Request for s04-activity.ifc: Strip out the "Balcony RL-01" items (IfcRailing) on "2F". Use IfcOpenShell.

First a look at what the model holds.

```python
import ifcopenshell
import ifcopenshell.util.element

model = ifcopenshell.open("s04-activity.ifc")
print(model.schema)
storey = next(s for s in model.by_type("IfcBuildingStorey") if s.Name == "2F")
railings = [e for e in ifcopenshell.util.element.get_decomposition(storey) if e.is_a("IfcRailing")]
seen = {}
for e in railings:
    element_type = ifcopenshell.util.element.get_type(e)
    name = element_type.Name if element_type not in (None, e) else None
    seen[name] = seen.get(name, 0) + 1
for name, count in sorted(seen.items(), key=str):
    print(count, "x", name)
```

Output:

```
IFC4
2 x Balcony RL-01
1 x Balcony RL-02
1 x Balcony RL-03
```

```python
import ifcopenshell
import ifcopenshell.api.root
import ifcopenshell.util.element

model = ifcopenshell.open("s04-activity.ifc")

storey = next(s for s in model.by_type("IfcBuildingStorey") if s.Name == "2F")
railings = [e for e in ifcopenshell.util.element.get_decomposition(storey) if e.is_a("IfcRailing")]
targets = [e for e in railings if (t := ifcopenshell.util.element.get_type(e)) not in (None, e) and t.Name == "Balcony RL-01"]

for e in targets:
    ifcopenshell.api.root.remove_product(model, product=e)
print(len(targets), "removed")

model.write("s04-activity_updated.ifc")
```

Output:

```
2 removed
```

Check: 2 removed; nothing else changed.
